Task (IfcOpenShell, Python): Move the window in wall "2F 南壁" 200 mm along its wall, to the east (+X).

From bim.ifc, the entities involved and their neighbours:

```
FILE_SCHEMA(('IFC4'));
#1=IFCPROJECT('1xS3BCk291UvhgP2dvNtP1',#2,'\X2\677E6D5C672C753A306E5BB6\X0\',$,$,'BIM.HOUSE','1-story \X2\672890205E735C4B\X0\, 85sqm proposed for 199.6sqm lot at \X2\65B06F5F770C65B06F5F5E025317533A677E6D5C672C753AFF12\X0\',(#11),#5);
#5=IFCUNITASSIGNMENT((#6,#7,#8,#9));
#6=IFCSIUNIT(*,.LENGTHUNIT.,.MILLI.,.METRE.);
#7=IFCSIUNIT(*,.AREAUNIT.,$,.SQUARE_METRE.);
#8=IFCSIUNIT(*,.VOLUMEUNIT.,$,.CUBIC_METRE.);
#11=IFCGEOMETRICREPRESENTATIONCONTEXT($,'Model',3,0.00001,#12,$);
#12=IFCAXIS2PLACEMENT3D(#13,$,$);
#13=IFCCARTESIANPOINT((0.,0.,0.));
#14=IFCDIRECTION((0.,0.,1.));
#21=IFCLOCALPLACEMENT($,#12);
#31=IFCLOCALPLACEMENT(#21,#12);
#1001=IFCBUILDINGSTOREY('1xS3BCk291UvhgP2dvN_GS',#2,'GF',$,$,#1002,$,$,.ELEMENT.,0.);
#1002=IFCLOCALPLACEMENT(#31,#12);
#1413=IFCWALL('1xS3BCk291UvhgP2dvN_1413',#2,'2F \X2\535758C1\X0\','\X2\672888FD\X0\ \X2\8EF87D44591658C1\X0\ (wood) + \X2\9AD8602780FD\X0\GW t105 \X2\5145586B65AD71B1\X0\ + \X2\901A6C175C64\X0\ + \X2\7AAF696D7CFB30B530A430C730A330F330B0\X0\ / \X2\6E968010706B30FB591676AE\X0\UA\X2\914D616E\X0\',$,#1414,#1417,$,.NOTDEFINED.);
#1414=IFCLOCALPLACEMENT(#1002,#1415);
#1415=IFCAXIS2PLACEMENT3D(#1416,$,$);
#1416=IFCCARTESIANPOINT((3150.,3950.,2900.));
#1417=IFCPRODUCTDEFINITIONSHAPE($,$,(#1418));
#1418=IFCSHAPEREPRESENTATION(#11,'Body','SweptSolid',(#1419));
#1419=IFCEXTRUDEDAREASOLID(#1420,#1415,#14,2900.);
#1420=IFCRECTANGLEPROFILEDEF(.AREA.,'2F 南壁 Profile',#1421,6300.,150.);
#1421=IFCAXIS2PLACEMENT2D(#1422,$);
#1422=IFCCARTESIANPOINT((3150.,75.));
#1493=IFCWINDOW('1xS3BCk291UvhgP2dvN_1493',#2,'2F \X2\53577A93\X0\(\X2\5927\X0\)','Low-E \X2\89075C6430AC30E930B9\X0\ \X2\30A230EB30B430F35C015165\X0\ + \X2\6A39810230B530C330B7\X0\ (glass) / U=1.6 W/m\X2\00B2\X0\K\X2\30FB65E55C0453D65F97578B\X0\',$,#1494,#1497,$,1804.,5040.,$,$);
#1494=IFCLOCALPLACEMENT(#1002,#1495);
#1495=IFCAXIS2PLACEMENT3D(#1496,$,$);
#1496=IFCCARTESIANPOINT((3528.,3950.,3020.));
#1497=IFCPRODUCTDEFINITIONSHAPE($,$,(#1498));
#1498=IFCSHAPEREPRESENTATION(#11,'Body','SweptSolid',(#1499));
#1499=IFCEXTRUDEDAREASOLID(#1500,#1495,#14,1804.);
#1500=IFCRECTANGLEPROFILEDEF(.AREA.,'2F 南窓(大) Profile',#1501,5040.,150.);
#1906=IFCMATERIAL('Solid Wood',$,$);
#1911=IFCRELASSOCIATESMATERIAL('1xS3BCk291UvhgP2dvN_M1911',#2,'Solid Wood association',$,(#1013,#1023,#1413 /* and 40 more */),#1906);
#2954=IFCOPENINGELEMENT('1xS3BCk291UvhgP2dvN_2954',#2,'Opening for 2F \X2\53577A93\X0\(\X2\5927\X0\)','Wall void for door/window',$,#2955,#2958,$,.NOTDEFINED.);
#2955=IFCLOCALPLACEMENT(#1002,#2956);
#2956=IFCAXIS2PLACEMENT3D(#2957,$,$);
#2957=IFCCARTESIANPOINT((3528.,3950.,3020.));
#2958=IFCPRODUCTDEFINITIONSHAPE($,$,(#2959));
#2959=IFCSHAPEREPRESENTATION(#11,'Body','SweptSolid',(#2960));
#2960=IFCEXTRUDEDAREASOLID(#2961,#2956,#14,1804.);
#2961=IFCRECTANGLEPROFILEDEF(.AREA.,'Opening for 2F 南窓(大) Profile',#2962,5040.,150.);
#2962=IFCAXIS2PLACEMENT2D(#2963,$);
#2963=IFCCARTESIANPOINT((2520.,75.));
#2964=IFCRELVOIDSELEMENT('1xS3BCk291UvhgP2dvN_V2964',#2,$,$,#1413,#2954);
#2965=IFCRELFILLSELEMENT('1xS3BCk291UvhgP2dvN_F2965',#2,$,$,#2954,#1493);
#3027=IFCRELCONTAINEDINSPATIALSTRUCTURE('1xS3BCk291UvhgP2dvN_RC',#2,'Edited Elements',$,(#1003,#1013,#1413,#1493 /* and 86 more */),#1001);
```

```python
import ifcopenshell
import ifcopenshell.api.geometry
import ifcopenshell.util.placement
import ifcopenshell.util.unit

model = ifcopenshell.open("bim.ifc")
unit_scale = ifcopenshell.util.unit.calculate_unit_scale(model)

window = model.by_guid("1xS3BCk291UvhgP2dvN_1493")
opening = window.FillsVoids[0].RelatingOpeningElement
wall = opening.VoidsElements[0].RelatingBuildingElement

wall_matrix = ifcopenshell.util.placement.get_local_placement(wall.ObjectPlacement)
shift = wall_matrix[:3, 0] * 0.2 / unit_scale
before = ifcopenshell.util.placement.get_local_placement(window.ObjectPlacement)[:3, 3].copy()

# The window is not placed relative to its opening, so move both.
for product in (opening, window):
    matrix = ifcopenshell.util.placement.get_local_placement(product.ObjectPlacement)
    matrix[:3, 3] += shift
    ifcopenshell.api.geometry.edit_object_placement(model, product=product, matrix=matrix, is_si=False)

after = ifcopenshell.util.placement.get_local_placement(window.ObjectPlacement)[:3, 3]
print("window moved by", (after - before).round(3) + 0.0)

model.write("bim_v2.ifc")
```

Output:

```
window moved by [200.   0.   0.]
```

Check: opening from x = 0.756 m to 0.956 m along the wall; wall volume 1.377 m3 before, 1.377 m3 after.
